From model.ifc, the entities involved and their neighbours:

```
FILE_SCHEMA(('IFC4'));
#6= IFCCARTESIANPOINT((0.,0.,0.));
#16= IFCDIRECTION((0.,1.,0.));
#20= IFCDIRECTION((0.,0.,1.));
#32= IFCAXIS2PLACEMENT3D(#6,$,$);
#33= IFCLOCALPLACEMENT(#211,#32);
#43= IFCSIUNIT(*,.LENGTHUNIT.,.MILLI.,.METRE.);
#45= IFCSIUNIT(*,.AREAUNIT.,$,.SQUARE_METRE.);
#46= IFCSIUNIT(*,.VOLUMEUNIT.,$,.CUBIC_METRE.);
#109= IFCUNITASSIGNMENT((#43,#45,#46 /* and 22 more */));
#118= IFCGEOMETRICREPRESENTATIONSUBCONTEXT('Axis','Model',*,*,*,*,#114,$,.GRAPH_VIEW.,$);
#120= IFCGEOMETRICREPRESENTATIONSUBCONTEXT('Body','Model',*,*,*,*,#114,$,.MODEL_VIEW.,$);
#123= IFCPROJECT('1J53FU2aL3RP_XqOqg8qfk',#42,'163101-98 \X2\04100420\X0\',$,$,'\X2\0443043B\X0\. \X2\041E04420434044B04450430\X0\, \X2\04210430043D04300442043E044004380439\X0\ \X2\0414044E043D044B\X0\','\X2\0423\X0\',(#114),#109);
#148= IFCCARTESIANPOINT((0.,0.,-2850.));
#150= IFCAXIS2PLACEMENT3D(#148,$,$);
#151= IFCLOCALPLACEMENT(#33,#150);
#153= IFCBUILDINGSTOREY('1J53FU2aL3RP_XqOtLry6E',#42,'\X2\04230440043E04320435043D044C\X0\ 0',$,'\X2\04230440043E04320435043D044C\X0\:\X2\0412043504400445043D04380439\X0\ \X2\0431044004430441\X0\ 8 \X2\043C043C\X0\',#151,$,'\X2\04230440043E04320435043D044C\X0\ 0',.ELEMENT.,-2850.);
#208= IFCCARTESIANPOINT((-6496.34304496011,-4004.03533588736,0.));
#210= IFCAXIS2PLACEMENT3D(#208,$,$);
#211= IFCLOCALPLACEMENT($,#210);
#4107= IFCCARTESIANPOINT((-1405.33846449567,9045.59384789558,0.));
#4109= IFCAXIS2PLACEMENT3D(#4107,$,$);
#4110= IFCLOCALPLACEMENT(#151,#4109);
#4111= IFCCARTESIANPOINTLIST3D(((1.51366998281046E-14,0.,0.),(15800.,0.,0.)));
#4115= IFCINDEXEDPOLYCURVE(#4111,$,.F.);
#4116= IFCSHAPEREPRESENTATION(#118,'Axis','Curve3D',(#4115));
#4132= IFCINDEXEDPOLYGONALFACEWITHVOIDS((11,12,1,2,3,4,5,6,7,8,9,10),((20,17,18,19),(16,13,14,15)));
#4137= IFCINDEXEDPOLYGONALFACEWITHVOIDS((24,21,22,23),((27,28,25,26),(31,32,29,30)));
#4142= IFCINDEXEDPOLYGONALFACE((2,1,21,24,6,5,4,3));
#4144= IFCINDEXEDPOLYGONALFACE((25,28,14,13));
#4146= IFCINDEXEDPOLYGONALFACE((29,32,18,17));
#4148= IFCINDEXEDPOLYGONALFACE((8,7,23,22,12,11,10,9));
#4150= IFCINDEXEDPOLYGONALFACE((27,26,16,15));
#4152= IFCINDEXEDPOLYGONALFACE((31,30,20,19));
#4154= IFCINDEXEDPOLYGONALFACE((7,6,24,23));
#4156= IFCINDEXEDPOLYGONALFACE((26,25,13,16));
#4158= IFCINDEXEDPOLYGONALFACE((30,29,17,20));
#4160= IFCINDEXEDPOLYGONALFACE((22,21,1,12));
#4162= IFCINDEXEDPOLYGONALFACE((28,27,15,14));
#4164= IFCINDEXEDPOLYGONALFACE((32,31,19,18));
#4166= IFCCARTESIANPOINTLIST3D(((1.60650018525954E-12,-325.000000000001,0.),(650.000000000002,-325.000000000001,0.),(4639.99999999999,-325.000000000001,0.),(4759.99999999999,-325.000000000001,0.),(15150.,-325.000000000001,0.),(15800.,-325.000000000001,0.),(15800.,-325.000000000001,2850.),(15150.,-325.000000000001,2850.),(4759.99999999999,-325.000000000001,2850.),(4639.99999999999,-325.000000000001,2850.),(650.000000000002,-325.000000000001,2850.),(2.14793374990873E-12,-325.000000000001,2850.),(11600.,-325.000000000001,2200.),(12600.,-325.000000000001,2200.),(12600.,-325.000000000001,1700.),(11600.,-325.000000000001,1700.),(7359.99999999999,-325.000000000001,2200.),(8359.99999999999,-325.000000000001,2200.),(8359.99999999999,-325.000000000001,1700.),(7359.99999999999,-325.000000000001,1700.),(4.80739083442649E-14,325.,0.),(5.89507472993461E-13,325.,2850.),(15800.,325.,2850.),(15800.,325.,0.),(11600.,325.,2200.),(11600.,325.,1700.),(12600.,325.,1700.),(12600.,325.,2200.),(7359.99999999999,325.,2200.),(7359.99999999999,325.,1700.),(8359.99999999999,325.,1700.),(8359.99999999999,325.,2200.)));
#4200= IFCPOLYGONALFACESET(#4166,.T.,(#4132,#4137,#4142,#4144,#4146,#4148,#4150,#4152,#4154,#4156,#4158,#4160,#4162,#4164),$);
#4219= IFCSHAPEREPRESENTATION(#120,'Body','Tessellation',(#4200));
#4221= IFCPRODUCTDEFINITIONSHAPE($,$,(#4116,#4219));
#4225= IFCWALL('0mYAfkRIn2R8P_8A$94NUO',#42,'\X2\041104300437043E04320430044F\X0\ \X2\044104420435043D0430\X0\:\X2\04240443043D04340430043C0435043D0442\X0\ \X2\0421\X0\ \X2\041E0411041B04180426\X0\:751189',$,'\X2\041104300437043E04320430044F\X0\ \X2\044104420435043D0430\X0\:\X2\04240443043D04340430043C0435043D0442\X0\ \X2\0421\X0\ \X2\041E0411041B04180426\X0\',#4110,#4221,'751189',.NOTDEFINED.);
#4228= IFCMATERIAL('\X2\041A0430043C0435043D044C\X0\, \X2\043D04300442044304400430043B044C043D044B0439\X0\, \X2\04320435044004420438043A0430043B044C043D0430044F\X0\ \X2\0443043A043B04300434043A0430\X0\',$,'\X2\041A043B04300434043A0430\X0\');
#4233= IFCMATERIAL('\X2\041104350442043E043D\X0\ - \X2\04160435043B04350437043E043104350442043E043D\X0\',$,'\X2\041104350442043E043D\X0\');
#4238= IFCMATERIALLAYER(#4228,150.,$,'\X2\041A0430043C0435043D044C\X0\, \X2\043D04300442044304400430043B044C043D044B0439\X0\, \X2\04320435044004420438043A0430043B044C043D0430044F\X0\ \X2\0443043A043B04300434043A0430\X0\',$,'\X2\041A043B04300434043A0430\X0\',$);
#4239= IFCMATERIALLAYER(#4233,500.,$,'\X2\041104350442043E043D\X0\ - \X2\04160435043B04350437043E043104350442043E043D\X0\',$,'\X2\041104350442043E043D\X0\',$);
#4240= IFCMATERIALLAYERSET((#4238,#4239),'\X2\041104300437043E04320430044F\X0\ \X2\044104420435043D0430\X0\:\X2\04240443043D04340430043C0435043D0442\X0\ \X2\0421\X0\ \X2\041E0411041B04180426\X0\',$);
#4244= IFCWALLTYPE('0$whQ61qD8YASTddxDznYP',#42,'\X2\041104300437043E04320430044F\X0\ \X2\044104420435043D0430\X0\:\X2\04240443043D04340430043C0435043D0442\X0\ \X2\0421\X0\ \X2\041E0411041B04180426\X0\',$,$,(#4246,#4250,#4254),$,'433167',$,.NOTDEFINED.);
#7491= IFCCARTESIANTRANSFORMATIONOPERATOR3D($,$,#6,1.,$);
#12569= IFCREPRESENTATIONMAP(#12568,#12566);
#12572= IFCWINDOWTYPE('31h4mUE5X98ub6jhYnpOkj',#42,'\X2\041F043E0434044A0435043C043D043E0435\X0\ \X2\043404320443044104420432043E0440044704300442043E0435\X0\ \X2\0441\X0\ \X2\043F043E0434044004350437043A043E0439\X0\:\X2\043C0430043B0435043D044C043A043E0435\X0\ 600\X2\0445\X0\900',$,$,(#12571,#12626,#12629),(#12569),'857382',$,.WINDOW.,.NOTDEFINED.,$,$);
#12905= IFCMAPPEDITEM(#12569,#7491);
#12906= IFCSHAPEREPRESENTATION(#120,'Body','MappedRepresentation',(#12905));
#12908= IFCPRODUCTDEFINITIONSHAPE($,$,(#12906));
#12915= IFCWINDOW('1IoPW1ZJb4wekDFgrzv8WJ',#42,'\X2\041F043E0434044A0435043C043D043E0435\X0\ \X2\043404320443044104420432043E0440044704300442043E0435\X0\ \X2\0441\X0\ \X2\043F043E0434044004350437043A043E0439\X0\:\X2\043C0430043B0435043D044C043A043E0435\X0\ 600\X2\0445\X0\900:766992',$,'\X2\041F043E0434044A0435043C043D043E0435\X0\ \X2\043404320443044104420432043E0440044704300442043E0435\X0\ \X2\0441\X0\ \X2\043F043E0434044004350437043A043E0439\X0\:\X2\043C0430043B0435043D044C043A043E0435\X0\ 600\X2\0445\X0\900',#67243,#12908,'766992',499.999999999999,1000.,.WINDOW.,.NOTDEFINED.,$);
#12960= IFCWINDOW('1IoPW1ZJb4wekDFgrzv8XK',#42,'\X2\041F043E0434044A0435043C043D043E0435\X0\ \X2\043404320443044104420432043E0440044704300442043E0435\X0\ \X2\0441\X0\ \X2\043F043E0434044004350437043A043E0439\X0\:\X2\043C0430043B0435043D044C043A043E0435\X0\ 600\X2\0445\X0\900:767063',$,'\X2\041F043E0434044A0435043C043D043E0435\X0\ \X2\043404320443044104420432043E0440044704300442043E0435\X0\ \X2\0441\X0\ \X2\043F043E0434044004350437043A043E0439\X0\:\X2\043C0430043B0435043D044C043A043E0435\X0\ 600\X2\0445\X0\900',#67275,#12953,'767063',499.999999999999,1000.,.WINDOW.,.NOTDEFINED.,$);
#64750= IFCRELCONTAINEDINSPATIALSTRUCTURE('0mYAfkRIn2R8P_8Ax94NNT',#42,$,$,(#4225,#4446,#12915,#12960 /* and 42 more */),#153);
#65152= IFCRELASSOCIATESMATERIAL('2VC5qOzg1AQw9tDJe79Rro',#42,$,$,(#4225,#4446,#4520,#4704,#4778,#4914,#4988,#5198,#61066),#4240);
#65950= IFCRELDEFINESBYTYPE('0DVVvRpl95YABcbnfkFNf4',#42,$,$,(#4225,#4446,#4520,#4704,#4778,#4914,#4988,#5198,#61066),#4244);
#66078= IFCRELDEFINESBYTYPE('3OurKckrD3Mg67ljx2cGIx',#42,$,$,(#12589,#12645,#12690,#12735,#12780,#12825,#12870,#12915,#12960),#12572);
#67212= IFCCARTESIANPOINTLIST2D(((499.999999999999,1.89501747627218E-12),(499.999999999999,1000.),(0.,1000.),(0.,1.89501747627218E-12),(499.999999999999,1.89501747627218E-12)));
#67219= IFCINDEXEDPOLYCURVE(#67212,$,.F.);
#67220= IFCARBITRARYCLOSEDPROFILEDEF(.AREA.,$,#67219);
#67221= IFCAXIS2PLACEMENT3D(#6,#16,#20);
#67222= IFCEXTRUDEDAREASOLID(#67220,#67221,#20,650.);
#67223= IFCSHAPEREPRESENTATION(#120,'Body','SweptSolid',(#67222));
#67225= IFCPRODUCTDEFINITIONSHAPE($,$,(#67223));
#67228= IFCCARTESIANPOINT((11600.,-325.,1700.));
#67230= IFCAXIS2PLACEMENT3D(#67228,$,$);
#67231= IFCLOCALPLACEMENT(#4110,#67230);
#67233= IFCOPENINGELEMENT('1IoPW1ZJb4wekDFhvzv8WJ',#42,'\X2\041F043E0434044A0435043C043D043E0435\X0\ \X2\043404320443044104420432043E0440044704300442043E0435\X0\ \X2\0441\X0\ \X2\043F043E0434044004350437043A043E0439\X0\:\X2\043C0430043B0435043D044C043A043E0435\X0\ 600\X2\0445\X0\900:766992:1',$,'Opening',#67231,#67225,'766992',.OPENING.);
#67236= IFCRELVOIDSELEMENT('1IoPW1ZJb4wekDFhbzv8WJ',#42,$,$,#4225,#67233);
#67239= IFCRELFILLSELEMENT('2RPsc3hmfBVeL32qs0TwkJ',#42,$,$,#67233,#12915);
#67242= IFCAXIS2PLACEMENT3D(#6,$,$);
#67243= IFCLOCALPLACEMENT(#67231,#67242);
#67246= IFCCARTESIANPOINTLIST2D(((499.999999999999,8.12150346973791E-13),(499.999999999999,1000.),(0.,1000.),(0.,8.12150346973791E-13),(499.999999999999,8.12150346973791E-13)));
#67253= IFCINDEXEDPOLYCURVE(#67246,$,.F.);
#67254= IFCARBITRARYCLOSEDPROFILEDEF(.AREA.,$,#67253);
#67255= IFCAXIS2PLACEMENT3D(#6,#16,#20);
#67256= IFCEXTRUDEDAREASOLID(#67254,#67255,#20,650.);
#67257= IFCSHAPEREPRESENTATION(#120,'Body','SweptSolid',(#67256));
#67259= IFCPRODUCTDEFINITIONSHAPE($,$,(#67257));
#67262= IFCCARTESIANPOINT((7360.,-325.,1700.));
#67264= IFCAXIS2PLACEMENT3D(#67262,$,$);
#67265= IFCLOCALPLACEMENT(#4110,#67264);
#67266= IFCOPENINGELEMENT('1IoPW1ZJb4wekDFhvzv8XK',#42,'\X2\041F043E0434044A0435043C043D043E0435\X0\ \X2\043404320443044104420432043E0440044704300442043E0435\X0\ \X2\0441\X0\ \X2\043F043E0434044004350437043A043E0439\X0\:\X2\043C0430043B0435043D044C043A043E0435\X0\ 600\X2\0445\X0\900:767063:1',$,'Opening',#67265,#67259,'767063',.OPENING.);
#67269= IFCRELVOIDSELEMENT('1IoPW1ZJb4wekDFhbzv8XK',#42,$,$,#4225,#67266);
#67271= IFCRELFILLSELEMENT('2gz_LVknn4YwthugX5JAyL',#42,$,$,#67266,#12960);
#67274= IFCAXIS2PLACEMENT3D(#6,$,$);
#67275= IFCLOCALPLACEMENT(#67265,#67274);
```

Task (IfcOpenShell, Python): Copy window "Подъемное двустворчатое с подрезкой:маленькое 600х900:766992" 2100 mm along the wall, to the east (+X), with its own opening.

```python
import ifcopenshell
import ifcopenshell.api.feature
import ifcopenshell.api.geometry
import ifcopenshell.api.root
import ifcopenshell.geom
import ifcopenshell.util.element
import ifcopenshell.util.placement
import ifcopenshell.util.shape
import ifcopenshell.util.unit

model = ifcopenshell.open("model.ifc")
unit_scale = ifcopenshell.util.unit.calculate_unit_scale(model)
settings = ifcopenshell.geom.settings()


def volume(element):
    """Net volume in cubic metres, openings subtracted."""
    shape = ifcopenshell.geom.create_shape(settings, element)
    return ifcopenshell.util.shape.get_volume(shape.geometry)


def reuse_history(source, copy):
    """copy_class also copies each property set's owner history, people and application; keep the originals."""
    for rel in copy.IsDefinedBy:
        if rel.is_a("IfcRelDefinesByProperties") and (history := rel.RelatingPropertyDefinition.OwnerHistory):
            rel.RelatingPropertyDefinition.OwnerHistory = source.OwnerHistory
            ifcopenshell.util.element.remove_deep2(model, history)


window = model.by_guid("1IoPW1ZJb4wekDFgrzv8WJ")
opening = window.FillsVoids[0].RelatingOpeningElement
wall = opening.VoidsElements[0].RelatingBuildingElement
before = volume(wall)
shift = ifcopenshell.util.placement.get_local_placement(wall.ObjectPlacement)[:3, 0] * 2.1 / unit_scale

# copy_class copies the void relationship, type, container and properties, but no geometry.
new_opening = ifcopenshell.api.root.copy_class(model, product=opening)
new_opening.Representation = ifcopenshell.util.element.copy_deep(
    model, opening.Representation, exclude=["IfcGeometricRepresentationContext", "IfcRepresentationMap"]
)
new_opening.Name = "Подъемное двустворчатое с подрезкой:маленькое 600х900"
new_opening.Tag = None
new_window = ifcopenshell.api.root.copy_class(model, product=window)
new_window.Representation = ifcopenshell.util.element.copy_deep(
    model, window.Representation, exclude=["IfcGeometricRepresentationContext", "IfcRepresentationMap"]
)
new_window.Name = "Подъемное двустворчатое с подрезкой:маленькое 600х900"
new_window.Tag = None
reuse_history(window, new_window)
ifcopenshell.api.feature.add_filling(model, opening=new_opening, element=new_window)

for old, new in ((opening, new_opening), (window, new_window)):
    matrix = ifcopenshell.util.placement.get_local_placement(old.ObjectPlacement)
    matrix[:3, 3] += shift
    ifcopenshell.api.geometry.edit_object_placement(model, product=new, matrix=matrix, is_si=False)

after = volume(wall)

print(f"wall volume {before:.3f} -> {after:.3f} m3")

model.write("model_updated.ifc")
```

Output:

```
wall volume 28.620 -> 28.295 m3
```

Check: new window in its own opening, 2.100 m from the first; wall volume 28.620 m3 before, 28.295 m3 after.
